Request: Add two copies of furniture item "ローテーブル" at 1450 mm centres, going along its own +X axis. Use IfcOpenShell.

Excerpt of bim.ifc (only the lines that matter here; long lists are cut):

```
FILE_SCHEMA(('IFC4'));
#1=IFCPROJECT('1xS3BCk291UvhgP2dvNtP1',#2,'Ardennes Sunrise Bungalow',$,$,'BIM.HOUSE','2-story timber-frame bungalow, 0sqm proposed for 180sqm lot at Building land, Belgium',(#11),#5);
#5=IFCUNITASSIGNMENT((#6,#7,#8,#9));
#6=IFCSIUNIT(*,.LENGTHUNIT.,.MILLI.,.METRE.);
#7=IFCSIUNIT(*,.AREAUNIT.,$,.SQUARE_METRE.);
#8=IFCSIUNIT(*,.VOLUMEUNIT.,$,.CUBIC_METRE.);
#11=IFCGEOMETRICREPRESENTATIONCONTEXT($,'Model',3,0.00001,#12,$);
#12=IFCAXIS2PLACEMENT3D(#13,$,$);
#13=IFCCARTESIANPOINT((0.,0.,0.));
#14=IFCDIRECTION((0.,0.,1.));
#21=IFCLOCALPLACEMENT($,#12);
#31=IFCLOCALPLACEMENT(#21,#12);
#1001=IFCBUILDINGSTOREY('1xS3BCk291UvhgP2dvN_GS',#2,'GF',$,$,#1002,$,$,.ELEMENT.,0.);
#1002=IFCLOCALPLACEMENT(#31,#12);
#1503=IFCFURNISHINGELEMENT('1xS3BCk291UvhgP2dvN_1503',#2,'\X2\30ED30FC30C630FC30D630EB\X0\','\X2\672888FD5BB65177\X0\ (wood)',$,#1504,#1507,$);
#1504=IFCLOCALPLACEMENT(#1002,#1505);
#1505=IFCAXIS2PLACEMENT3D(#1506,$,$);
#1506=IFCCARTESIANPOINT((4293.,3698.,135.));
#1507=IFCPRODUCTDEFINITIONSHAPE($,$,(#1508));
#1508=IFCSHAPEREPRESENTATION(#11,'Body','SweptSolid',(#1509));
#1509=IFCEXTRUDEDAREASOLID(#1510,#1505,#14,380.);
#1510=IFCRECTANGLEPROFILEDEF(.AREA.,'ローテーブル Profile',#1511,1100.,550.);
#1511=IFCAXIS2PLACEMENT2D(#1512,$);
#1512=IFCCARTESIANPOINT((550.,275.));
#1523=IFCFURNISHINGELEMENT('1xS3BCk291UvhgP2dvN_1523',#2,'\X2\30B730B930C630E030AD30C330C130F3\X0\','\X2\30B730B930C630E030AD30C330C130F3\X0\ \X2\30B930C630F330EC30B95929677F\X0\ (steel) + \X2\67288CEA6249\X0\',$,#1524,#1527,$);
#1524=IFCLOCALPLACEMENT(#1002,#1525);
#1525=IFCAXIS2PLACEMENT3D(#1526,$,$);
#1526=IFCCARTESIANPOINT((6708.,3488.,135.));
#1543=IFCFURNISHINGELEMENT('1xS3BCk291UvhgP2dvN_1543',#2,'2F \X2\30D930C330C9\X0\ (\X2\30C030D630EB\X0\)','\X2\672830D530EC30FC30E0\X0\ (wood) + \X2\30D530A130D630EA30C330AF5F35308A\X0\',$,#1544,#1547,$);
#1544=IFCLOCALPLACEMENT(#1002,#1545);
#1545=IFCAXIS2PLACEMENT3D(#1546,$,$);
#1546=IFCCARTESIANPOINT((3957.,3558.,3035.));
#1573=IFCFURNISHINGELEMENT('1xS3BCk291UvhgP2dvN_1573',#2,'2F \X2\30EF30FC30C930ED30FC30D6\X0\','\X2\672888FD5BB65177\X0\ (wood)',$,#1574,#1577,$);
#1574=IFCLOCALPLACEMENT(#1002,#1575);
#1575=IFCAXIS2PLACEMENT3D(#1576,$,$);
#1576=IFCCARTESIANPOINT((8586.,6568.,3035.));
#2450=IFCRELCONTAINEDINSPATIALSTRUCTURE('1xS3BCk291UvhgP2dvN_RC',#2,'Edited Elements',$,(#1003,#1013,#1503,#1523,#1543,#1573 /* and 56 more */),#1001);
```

```python
import ifcopenshell
import ifcopenshell.api.geometry
import ifcopenshell.api.root
import ifcopenshell.util.element
import ifcopenshell.util.placement

model = ifcopenshell.open("bim.ifc")


def reuse_history(source, copy):
    """copy_class also copies each property set's owner history, people and application; keep the originals."""
    for rel in copy.IsDefinedBy:
        if rel.is_a("IfcRelDefinesByProperties") and (history := rel.RelatingPropertyDefinition.OwnerHistory):
            rel.RelatingPropertyDefinition.OwnerHistory = source.OwnerHistory
            ifcopenshell.util.element.remove_deep2(model, history)


source = model.by_guid("1xS3BCk291UvhgP2dvN_1503")
base = ifcopenshell.util.placement.get_local_placement(source.ObjectPlacement)
step = base[:3, 0] * 1450.0

for i in range(1, 3):
    copy = ifcopenshell.api.root.copy_class(model, product=source)
    copy.Representation = ifcopenshell.util.element.copy_deep(
        model, source.Representation, exclude=["IfcGeometricRepresentationContext", "IfcRepresentationMap"]
    )
    reuse_history(source, copy)
    matrix = base.copy()
    matrix[:3, 3] += i * step
    print("added at", matrix[:3, 3].round(3) + 0.0)
    ifcopenshell.api.geometry.edit_object_placement(model, product=copy, matrix=matrix, is_si=False)

model.write("bim_rev.ifc")
```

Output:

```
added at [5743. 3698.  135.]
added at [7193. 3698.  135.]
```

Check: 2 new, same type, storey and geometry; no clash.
